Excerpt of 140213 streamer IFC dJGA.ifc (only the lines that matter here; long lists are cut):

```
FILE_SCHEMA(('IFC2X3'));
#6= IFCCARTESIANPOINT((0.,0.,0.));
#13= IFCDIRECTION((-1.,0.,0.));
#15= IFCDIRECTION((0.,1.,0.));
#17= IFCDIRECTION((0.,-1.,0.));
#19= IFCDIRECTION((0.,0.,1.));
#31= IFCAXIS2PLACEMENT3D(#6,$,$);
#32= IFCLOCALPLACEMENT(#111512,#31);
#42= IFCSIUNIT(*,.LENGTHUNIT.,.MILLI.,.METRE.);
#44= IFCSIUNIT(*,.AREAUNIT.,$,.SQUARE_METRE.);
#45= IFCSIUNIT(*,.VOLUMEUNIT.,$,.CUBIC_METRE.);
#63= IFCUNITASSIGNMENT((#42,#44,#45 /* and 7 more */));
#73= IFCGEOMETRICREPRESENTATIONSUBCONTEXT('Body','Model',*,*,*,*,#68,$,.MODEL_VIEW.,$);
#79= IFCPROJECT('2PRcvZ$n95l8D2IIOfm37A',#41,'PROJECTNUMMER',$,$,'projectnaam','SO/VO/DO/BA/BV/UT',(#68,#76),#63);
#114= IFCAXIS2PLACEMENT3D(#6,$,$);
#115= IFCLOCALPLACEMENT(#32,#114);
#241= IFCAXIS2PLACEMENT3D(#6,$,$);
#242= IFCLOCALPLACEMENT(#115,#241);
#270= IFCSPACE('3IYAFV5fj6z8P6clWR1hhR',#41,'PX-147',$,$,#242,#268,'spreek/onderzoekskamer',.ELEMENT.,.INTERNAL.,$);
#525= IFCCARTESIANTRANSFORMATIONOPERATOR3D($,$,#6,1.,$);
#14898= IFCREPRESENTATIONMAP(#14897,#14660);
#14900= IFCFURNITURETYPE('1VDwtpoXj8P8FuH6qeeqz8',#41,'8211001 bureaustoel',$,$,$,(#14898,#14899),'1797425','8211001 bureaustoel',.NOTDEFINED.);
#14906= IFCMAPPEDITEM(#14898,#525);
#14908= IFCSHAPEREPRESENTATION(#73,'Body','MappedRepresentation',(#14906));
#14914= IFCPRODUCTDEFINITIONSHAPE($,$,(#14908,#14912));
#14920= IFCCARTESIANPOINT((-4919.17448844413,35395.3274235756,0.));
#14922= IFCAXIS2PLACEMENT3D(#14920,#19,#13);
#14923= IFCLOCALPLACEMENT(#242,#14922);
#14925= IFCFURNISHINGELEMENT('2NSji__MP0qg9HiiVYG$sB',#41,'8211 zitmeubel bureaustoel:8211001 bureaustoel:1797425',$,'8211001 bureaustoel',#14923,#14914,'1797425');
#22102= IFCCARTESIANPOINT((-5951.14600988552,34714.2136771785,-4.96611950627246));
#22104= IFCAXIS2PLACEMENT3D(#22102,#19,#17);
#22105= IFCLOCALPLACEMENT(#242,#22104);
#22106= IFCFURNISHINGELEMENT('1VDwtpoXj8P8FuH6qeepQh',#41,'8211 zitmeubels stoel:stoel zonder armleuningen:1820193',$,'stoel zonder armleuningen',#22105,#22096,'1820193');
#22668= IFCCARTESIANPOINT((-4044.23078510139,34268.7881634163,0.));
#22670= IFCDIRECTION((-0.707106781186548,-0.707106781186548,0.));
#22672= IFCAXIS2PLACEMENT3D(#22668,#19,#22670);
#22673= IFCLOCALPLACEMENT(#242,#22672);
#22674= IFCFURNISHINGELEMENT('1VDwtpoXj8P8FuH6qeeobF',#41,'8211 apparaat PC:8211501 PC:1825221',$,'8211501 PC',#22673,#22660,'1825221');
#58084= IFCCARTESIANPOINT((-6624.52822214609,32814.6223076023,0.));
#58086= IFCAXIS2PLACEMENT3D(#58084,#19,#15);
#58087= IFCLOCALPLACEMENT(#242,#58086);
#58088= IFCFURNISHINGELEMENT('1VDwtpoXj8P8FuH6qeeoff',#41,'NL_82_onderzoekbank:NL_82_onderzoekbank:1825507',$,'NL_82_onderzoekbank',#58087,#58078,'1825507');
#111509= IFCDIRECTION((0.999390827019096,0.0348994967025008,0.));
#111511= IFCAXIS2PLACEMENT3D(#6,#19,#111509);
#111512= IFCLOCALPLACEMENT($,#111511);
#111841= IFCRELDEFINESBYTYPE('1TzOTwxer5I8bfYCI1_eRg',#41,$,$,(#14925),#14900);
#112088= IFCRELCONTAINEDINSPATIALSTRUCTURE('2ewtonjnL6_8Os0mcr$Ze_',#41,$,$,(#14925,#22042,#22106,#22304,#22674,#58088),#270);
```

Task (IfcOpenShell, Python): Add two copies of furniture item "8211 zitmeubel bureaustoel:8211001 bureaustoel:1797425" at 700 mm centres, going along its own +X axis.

```python
import ifcopenshell
import ifcopenshell.api.geometry
import ifcopenshell.api.root
import ifcopenshell.util.element
import ifcopenshell.util.placement
import ifcopenshell.util.unit

model = ifcopenshell.open("140213 streamer IFC dJGA.ifc")
unit_scale = ifcopenshell.util.unit.calculate_unit_scale(model)


def reuse_history(source, copy):
    """copy_class also copies each property set's owner history, people and application; keep the originals."""
    for rel in copy.IsDefinedBy:
        if rel.is_a("IfcRelDefinesByProperties") and (history := rel.RelatingPropertyDefinition.OwnerHistory):
            rel.RelatingPropertyDefinition.OwnerHistory = source.OwnerHistory
            ifcopenshell.util.element.remove_deep2(model, history)


source = model.by_guid("2NSji__MP0qg9HiiVYG$sB")
base = ifcopenshell.util.placement.get_local_placement(source.ObjectPlacement)
step = base[:3, 0] * 0.7 / unit_scale

for i in range(1, 3):
    copy = ifcopenshell.api.root.copy_class(model, product=source)
    copy.Representation = ifcopenshell.util.element.copy_deep(
        model, source.Representation, exclude=["IfcGeometricRepresentationContext", "IfcRepresentationMap"]
    )
    copy.Name = "8211 zitmeubel bureaustoel:8211001 bureaustoel"
    copy.Tag = None
    reuse_history(source, copy)
    matrix = base.copy()
    matrix[:3, 3] += i * step
    print("added at", matrix[:3, 3].round(3) + 0.0)
    ifcopenshell.api.geometry.edit_object_placement(model, product=copy, matrix=matrix, is_si=False)

model.write("140213 streamer IFC dJGA-out.ifc")
```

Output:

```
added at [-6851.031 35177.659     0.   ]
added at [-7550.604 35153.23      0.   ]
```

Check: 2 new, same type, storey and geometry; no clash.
